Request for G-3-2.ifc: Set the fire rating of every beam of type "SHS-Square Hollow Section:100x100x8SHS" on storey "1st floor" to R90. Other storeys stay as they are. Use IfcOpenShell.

First a look at what the model holds.

```python
import ifcopenshell
import ifcopenshell.util.element

model = ifcopenshell.open("G-3-2.ifc")
print(model.schema)
storey = next(s for s in model.by_type("IfcBuildingStorey") if s.Name == "1st floor")
beams = [e for e in ifcopenshell.util.element.get_decomposition(storey) if e.is_a("IfcBeam")]
seen = {}
for e in beams:
    element_type = ifcopenshell.util.element.get_type(e)
    key = (element_type.Name if element_type != e and element_type else None, ifcopenshell.util.element.get_pset(e, "Pset_BeamCommon", "FireRating"))
    seen[key] = seen.get(key, 0) + 1
for (name, value), count in sorted(seen.items(), key=str):
    print(count, "x", name, "|", value)
```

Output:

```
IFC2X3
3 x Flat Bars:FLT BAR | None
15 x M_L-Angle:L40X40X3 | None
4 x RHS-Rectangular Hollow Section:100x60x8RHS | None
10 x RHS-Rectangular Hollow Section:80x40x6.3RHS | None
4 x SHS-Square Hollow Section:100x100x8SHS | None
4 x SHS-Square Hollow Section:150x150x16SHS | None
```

```python
import ifcopenshell
import ifcopenshell.api.pset
import ifcopenshell.util.element

model = ifcopenshell.open("G-3-2.ifc")

storey = next(s for s in model.by_type("IfcBuildingStorey") if s.Name == "1st floor")
beams = [e for e in ifcopenshell.util.element.get_decomposition(storey) if e.is_a("IfcBeam")]

count = 0
for e in beams:
    element_type = ifcopenshell.util.element.get_type(e)
    if element_type in (None, e) or element_type.Name != "SHS-Square Hollow Section:100x100x8SHS":
        continue
    # add_pset returns the element's existing set when there is one.
    pset = ifcopenshell.api.pset.add_pset(model, product=e, name="Pset_BeamCommon")
    ifcopenshell.api.pset.edit_pset(model, pset=pset, properties={"FireRating": "R90"})
    count += 1

print(count, "beams updated")

model.write("G-3-2_updated.ifc")
```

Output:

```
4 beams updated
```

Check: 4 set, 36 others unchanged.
